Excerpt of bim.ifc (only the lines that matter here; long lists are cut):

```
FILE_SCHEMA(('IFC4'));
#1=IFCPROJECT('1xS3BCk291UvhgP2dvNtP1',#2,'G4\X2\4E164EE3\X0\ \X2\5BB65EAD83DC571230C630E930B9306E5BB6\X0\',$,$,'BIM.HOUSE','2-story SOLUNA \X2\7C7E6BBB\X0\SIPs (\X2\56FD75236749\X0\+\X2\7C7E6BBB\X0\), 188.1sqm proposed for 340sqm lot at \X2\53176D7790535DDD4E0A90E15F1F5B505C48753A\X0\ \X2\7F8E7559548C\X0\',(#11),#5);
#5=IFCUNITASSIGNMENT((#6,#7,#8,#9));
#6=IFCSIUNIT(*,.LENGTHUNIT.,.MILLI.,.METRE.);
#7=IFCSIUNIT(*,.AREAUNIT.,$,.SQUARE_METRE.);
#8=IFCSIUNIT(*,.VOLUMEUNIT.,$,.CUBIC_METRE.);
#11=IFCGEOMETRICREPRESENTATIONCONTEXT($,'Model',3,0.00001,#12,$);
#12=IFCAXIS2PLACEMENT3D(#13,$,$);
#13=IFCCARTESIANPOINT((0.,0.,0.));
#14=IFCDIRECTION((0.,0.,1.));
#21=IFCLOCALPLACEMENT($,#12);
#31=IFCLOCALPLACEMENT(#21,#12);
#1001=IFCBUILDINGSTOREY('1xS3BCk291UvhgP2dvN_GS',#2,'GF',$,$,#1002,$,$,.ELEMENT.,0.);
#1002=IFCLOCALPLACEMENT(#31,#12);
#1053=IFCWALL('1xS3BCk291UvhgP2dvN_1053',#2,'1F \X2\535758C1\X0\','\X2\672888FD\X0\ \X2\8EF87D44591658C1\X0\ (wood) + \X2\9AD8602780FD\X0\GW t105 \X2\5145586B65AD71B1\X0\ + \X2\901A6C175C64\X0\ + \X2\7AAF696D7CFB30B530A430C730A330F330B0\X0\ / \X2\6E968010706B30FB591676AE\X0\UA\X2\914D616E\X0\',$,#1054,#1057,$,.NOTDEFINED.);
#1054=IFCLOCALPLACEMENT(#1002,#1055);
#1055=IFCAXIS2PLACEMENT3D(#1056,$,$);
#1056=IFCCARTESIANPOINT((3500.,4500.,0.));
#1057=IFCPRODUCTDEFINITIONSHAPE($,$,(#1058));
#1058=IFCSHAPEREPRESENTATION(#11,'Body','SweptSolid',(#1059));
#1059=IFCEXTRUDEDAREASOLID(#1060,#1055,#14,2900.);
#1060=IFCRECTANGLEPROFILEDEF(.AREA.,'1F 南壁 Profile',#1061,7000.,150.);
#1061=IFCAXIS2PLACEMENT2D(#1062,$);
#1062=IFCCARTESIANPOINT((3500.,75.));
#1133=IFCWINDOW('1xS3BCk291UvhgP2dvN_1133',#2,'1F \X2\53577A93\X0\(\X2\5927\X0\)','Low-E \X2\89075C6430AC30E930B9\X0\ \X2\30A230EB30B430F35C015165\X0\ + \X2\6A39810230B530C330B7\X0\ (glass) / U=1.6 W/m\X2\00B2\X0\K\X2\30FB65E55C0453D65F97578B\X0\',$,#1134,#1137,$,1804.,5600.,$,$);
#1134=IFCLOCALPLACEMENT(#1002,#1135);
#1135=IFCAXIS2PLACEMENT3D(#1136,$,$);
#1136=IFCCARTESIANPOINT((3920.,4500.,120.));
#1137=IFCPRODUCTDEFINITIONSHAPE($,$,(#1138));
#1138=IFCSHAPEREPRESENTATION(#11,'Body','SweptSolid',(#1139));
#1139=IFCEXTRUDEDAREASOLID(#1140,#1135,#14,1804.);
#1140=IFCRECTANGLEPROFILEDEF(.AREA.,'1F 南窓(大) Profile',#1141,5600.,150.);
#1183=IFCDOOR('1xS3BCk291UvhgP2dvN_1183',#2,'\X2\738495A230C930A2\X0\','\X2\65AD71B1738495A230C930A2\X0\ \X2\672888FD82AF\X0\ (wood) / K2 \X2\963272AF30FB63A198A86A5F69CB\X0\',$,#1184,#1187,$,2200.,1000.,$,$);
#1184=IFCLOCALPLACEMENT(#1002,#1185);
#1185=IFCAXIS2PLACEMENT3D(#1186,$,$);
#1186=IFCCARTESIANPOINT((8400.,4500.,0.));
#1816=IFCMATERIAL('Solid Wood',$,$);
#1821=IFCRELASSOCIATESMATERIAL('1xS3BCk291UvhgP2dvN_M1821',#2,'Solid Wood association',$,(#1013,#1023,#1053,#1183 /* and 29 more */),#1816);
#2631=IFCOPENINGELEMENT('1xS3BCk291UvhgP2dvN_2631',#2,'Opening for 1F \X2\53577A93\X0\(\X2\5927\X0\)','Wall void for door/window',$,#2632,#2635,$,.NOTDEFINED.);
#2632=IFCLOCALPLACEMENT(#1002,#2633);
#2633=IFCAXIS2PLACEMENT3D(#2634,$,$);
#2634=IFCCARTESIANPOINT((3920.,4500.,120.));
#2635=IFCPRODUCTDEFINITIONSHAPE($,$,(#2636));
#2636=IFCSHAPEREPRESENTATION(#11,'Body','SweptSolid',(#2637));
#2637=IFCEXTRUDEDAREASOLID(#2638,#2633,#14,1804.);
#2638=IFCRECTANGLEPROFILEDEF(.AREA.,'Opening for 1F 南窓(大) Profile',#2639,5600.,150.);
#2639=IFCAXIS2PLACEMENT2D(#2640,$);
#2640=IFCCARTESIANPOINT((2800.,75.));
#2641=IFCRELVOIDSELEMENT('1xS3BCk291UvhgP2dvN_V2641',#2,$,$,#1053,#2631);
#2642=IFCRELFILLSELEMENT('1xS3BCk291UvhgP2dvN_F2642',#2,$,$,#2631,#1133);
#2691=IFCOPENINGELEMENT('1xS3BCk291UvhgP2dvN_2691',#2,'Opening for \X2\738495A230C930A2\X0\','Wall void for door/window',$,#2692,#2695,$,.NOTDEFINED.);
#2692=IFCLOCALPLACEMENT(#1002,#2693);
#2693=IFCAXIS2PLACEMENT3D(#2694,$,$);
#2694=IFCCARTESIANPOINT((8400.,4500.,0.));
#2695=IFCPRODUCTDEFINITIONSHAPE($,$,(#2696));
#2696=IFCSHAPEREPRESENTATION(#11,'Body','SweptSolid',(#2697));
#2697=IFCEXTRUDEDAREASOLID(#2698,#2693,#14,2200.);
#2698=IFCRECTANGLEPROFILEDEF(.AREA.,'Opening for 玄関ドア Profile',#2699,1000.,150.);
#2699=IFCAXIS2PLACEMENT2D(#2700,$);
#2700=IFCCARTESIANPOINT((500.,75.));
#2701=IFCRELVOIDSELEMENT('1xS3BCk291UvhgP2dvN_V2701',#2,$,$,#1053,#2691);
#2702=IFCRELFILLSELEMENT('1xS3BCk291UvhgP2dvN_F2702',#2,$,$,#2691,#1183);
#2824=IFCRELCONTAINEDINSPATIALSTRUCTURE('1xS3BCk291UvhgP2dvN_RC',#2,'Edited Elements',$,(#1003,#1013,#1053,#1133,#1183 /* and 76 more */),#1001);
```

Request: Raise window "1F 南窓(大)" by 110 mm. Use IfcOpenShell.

```python
import numpy as np
import ifcopenshell
import ifcopenshell.api.geometry
import ifcopenshell.util.placement
import ifcopenshell.util.unit

model = ifcopenshell.open("bim.ifc")
unit_scale = ifcopenshell.util.unit.calculate_unit_scale(model)

window = model.by_guid("1xS3BCk291UvhgP2dvN_1133")
opening = window.FillsVoids[0].RelatingOpeningElement
dz = 0.11 / unit_scale

shift = np.array([0.0, 0.0, dz])
# The window is not placed relative to its opening, so move both.
for product in (opening, window):
    matrix = ifcopenshell.util.placement.get_local_placement(product.ObjectPlacement)
    matrix[:3, 3] += shift
    ifcopenshell.api.geometry.edit_object_placement(model, product=product, matrix=matrix, is_si=False)

print(f"moved by {dz * unit_scale:+.3f} m")

model.write("bim_rev.ifc")
```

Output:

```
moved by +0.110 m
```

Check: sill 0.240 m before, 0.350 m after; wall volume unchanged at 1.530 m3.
